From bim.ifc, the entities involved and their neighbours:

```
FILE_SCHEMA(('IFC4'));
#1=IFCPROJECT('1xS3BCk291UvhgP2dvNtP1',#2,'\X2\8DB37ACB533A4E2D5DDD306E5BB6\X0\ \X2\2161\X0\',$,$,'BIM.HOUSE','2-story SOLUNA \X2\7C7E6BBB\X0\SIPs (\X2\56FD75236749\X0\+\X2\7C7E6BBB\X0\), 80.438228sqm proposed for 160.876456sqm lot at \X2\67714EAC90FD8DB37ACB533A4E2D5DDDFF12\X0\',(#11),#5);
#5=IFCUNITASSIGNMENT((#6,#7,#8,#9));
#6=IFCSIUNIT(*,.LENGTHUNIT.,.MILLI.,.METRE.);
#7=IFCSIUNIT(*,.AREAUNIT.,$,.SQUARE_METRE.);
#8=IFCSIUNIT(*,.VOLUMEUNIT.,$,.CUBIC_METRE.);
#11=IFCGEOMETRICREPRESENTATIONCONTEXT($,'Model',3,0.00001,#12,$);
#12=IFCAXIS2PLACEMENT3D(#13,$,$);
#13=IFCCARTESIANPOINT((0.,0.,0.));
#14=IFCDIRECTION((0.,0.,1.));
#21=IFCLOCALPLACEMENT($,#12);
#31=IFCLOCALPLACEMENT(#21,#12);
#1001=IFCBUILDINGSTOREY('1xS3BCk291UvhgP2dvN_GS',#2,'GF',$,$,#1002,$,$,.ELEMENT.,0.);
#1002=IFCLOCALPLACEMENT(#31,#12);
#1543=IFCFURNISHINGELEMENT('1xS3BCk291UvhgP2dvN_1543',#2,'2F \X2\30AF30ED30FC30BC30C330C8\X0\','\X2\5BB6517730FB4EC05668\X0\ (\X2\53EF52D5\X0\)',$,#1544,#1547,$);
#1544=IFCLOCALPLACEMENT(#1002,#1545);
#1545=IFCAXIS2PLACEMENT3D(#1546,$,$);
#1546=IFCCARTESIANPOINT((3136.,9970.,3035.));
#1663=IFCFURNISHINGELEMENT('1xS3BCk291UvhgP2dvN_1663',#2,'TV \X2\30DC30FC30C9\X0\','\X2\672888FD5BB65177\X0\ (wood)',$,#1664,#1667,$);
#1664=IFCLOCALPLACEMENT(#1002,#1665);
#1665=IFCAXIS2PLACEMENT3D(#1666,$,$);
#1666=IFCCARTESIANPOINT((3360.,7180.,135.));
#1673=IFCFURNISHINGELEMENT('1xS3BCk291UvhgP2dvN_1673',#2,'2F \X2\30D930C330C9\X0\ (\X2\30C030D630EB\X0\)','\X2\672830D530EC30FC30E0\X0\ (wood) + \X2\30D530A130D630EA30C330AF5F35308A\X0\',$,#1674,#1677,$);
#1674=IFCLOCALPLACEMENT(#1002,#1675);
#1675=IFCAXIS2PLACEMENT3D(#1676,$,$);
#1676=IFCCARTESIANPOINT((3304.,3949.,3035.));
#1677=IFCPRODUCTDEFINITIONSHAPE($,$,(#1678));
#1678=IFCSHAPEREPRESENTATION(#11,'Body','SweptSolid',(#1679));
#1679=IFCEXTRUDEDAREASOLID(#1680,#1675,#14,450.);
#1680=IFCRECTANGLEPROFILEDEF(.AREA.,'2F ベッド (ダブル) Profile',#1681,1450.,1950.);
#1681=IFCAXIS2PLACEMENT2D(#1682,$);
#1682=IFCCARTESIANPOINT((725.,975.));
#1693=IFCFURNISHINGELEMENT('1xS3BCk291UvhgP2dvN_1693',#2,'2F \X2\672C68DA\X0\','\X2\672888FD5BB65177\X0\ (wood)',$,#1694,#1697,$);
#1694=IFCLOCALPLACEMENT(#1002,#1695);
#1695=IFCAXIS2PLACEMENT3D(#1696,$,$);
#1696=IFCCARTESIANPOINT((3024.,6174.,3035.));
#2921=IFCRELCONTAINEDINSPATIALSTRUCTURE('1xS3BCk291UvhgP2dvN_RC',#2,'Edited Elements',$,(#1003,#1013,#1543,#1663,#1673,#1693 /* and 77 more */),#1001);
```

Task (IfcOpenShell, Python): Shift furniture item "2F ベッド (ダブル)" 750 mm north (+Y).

```python
import ifcopenshell
import ifcopenshell.api.geometry
import ifcopenshell.util.placement
import ifcopenshell.util.unit

model = ifcopenshell.open("bim.ifc")
unit_scale = ifcopenshell.util.unit.calculate_unit_scale(model)

item = model.by_id(1673)
matrix = ifcopenshell.util.placement.get_local_placement(item.ObjectPlacement)
matrix[1, 3] += 0.75 / unit_scale
ifcopenshell.api.geometry.edit_object_placement(model, product=item, matrix=matrix, is_si=False)

print(ifcopenshell.util.placement.get_local_placement(item.ObjectPlacement).round(3) + 0.0)

model.write("bim_edited.ifc")
```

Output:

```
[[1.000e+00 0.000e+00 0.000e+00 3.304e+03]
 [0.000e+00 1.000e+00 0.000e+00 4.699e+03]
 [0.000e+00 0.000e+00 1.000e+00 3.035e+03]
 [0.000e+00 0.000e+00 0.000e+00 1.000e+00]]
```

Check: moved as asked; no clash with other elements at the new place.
